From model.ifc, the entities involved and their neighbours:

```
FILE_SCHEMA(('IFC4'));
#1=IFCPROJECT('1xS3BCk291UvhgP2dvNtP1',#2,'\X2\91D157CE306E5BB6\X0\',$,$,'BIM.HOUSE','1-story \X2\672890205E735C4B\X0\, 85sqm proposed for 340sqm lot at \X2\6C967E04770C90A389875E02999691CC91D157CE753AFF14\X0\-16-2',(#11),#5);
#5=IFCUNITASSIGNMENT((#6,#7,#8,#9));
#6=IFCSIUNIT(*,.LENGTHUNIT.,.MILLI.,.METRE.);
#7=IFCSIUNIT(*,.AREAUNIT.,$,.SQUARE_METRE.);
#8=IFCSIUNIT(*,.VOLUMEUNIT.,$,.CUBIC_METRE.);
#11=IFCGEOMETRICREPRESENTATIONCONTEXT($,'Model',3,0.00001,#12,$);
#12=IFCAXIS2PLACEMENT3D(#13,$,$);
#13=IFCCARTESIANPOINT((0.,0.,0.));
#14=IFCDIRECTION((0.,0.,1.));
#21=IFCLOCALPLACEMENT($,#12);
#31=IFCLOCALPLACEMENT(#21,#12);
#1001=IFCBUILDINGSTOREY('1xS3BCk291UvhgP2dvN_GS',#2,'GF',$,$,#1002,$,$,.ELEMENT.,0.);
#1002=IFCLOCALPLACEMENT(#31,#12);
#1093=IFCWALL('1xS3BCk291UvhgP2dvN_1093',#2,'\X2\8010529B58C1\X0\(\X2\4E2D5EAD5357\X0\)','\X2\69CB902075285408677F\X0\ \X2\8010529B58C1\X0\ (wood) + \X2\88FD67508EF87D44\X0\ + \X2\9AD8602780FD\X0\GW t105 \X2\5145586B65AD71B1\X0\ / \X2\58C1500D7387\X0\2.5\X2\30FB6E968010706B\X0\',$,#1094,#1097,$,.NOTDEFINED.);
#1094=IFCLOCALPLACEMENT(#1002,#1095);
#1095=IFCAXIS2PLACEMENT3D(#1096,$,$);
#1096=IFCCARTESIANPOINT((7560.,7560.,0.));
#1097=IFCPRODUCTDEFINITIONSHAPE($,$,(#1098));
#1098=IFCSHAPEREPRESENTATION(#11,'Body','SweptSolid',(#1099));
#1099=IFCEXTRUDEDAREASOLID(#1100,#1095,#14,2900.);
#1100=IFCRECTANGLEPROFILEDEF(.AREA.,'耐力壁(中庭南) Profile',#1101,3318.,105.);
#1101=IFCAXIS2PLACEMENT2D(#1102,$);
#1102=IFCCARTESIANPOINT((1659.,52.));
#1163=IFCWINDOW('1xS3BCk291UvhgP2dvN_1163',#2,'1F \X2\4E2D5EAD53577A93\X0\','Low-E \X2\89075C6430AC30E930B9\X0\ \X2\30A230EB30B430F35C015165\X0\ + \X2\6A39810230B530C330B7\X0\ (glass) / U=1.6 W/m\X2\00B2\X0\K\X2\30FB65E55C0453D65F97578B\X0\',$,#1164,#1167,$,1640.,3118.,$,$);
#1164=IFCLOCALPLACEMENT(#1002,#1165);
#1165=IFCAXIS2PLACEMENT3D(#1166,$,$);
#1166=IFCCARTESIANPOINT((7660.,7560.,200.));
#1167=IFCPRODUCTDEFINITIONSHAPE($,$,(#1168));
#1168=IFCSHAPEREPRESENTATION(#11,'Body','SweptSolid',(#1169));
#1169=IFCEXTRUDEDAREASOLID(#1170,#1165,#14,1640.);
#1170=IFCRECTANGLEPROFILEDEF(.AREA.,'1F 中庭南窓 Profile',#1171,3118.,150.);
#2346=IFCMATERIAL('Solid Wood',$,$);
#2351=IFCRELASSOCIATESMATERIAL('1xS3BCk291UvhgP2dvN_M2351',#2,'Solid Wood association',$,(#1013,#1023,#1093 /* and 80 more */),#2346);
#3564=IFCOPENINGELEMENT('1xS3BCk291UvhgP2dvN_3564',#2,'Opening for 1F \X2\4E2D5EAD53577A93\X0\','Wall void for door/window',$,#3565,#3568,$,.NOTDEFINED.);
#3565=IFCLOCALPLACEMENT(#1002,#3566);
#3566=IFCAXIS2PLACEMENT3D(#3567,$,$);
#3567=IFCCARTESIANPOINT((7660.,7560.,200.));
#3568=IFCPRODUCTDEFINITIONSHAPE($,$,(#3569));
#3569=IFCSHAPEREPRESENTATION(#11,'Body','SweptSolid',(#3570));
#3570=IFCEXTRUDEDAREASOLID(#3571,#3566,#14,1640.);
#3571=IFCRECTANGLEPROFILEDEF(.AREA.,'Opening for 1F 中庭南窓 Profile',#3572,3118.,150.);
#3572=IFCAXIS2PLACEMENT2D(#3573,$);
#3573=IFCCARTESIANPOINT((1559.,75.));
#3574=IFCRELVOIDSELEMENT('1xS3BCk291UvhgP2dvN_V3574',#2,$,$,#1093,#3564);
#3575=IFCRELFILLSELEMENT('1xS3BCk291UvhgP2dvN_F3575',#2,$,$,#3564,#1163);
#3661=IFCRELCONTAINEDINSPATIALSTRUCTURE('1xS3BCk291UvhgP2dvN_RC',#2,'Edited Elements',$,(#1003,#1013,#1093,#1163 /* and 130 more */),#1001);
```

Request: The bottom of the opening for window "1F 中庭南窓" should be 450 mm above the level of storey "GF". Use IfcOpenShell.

```python
import numpy as np
import ifcopenshell
import ifcopenshell.api.geometry
import ifcopenshell.geom
import ifcopenshell.util.element
import ifcopenshell.util.placement
import ifcopenshell.util.shape
import ifcopenshell.util.unit

model = ifcopenshell.open("model.ifc")
unit_scale = ifcopenshell.util.unit.calculate_unit_scale(model)

window = model.by_guid("1xS3BCk291UvhgP2dvN_1163")
opening = window.FillsVoids[0].RelatingOpeningElement
storey = ifcopenshell.util.element.get_container(window, ifc_class="IfcBuildingStorey")
level = ifcopenshell.util.placement.get_local_placement(storey.ObjectPlacement)[2, 3]

# The opening's origin need not be at the sill, so measure its lowest point.
shape = ifcopenshell.geom.create_shape(ifcopenshell.geom.settings(), opening)
bottom = ifcopenshell.util.shape.get_shape_bottom_elevation(shape, shape.geometry) / unit_scale
dz = level + 0.45 / unit_scale - bottom

shift = np.array([0.0, 0.0, dz])
# The window is not placed relative to its opening, so move both.
for product in (opening, window):
    matrix = ifcopenshell.util.placement.get_local_placement(product.ObjectPlacement)
    matrix[:3, 3] += shift
    ifcopenshell.api.geometry.edit_object_placement(model, product=product, matrix=matrix, is_si=False)

print(f"moved by {dz * unit_scale:+.3f} m")

model.write("model_edited.ifc")
```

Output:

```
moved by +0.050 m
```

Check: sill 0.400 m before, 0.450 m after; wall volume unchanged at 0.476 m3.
